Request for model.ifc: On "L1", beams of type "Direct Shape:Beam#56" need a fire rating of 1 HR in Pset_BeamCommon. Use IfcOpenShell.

First a look at what the model holds.

```python
import ifcopenshell
import ifcopenshell.util.element

model = ifcopenshell.open("model.ifc")
print(model.schema)
storey = next(s for s in model.by_type("IfcBuildingStorey") if s.Name == "L1")
beams = [e for e in ifcopenshell.util.element.get_decomposition(storey) if e.is_a("IfcBeam")]
seen = {}
for e in beams:
    element_type = ifcopenshell.util.element.get_type(e)
    key = (element_type.Name if element_type != e and element_type else None, ifcopenshell.util.element.get_pset(e, "Pset_BeamCommon", "FireRating"))
    seen[key] = seen.get(key, 0) + 1
for (name, value), count in sorted(seen.items(), key=str):
    print(count, "x", name, "|", value)
```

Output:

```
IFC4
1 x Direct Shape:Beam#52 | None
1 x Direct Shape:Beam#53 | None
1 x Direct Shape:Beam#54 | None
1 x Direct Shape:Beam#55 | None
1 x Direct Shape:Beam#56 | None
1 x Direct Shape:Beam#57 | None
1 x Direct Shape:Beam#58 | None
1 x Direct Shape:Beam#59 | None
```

```python
import ifcopenshell
import ifcopenshell.api.pset
import ifcopenshell.util.element

model = ifcopenshell.open("model.ifc")

storey = next(s for s in model.by_type("IfcBuildingStorey") if s.Name == "L1")
beams = [e for e in ifcopenshell.util.element.get_decomposition(storey) if e.is_a("IfcBeam")]

count = 0
for e in beams:
    element_type = ifcopenshell.util.element.get_type(e)
    if element_type in (None, e) or element_type.Name != "Direct Shape:Beam#56":
        continue
    # add_pset returns the element's existing set when there is one.
    pset = ifcopenshell.api.pset.add_pset(model, product=e, name="Pset_BeamCommon")
    ifcopenshell.api.pset.edit_pset(model, pset=pset, properties={"FireRating": "1 HR"})
    count += 1

print(count, "beams updated")

model.write("model_updated.ifc")
```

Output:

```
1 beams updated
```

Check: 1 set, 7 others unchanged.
